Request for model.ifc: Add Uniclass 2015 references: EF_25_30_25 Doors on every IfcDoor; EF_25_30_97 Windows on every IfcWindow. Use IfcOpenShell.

First a look at what the model holds.

```python
import ifcopenshell

model = ifcopenshell.open("model.ifc")
print(model.schema)
print("classifications:", [c.Name for c in model.by_type("IfcClassification")])
for ifc_class in ("IfcDoor", "IfcRoof", "IfcStair", "IfcWall", "IfcWindow"):
    print(ifc_class, len(model.by_type(ifc_class)))
```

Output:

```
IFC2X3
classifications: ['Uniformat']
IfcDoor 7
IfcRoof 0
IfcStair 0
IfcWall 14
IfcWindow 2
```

```python
import ifcopenshell
import ifcopenshell.api.classification

model = ifcopenshell.open("model.ifc")

# IFC2X3 requires Source and Edition and has no link from the project to the system.
system = model.create_entity("IfcClassification", Source="NBS", Edition="2015", Name="Uniclass 2015")

codes = {
    "IfcDoor": ("EF_25_30_25", "Doors"),
    "IfcWindow": ("EF_25_30_97", "Windows"),
}
for ifc_class, (code, name) in codes.items():
    products = model.by_type(ifc_class)
    ifcopenshell.api.classification.add_reference(
        model, products=products, classification=system, identification=code, name=name
    )
    print(code, len(products))

model.write("model_edited.ifc")
```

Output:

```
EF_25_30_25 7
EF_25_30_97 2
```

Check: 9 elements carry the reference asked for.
